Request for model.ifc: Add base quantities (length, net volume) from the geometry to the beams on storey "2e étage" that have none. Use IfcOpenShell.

First a look at what the model holds.

```python
import ifcopenshell
import ifcopenshell.util.element
import ifcopenshell.util.unit

model = ifcopenshell.open("model.ifc")
print(model.schema)
for unit_type in ("LENGTHUNIT", "AREAUNIT", "VOLUMEUNIT"):
    print(unit_type, ifcopenshell.util.unit.calculate_unit_scale(model, unit_type))
storey = next(s for s in model.by_type("IfcBuildingStorey") if s.Name == "2e étage")
beams = [e for e in ifcopenshell.util.element.get_decomposition(storey) if e.is_a("IfcBeam")]
for e in sorted(beams, key=lambda e: e.id()):
    print(e.id(), e.is_a(), e.Name, list(ifcopenshell.util.element.get_psets(e, qtos_only=True)), sep=" | ")
```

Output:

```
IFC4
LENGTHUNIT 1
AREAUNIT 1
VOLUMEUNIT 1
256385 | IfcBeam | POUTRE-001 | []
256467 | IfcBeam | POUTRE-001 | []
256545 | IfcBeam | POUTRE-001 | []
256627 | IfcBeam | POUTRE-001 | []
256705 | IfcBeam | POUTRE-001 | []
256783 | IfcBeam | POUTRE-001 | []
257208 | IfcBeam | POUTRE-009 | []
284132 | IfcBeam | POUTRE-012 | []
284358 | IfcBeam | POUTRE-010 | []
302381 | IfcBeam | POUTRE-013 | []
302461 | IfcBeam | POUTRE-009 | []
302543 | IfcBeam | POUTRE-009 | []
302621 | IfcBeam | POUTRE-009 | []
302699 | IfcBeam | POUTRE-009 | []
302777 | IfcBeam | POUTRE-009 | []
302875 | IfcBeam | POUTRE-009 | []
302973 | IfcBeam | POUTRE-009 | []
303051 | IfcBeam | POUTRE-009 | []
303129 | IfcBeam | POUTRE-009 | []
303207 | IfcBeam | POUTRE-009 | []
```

```python
import ifcopenshell
import ifcopenshell.api.pset
import ifcopenshell.geom
import ifcopenshell.util.element
import ifcopenshell.util.shape
import ifcopenshell.util.unit

model = ifcopenshell.open("model.ifc")
unit_scale = ifcopenshell.util.unit.calculate_unit_scale(model)
volume_scale = ifcopenshell.util.unit.calculate_unit_scale(model, "VOLUMEUNIT")
settings = ifcopenshell.geom.settings()

storey = next(s for s in model.by_type("IfcBuildingStorey") if s.Name == "2e étage")
beams = [e for e in ifcopenshell.util.element.get_decomposition(storey) if e.is_a("IfcBeam")]

for e in sorted(beams, key=lambda e: e.id()):
    if ifcopenshell.util.element.get_psets(e, qtos_only=True, should_inherit=False):
        continue
    # Geometry comes back in metres, in the element's own axes.
    shape = ifcopenshell.geom.create_shape(settings, e)
    values = {
        "Length": ifcopenshell.util.shape.get_max_xyz(shape.geometry) / unit_scale,
        "NetVolume": ifcopenshell.util.shape.get_volume(shape.geometry) / volume_scale,
    }
    qto = ifcopenshell.api.pset.add_qto(model, product=e, name="Qto_BeamBaseQuantities")
    ifcopenshell.api.pset.edit_qto(model, qto=qto, properties=values)
    print(e.id(), {k: round(v, 3) for k, v in values.items()})

model.write("model-out.ifc")
```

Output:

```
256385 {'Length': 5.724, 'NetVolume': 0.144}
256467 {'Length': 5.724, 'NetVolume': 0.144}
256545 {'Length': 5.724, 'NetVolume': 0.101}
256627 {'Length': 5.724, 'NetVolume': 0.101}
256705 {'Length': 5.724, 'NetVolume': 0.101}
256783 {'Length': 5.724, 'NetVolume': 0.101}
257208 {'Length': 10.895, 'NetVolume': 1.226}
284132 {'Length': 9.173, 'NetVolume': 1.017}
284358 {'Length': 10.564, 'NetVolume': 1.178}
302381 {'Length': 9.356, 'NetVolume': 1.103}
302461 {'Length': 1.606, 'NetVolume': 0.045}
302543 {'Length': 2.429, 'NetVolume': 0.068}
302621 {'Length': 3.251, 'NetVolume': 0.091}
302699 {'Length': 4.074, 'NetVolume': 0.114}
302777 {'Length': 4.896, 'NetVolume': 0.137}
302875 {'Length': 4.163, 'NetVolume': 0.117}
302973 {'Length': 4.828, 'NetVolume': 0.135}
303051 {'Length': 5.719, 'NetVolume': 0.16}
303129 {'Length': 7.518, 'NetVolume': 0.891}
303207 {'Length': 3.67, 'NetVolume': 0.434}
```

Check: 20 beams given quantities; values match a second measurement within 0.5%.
